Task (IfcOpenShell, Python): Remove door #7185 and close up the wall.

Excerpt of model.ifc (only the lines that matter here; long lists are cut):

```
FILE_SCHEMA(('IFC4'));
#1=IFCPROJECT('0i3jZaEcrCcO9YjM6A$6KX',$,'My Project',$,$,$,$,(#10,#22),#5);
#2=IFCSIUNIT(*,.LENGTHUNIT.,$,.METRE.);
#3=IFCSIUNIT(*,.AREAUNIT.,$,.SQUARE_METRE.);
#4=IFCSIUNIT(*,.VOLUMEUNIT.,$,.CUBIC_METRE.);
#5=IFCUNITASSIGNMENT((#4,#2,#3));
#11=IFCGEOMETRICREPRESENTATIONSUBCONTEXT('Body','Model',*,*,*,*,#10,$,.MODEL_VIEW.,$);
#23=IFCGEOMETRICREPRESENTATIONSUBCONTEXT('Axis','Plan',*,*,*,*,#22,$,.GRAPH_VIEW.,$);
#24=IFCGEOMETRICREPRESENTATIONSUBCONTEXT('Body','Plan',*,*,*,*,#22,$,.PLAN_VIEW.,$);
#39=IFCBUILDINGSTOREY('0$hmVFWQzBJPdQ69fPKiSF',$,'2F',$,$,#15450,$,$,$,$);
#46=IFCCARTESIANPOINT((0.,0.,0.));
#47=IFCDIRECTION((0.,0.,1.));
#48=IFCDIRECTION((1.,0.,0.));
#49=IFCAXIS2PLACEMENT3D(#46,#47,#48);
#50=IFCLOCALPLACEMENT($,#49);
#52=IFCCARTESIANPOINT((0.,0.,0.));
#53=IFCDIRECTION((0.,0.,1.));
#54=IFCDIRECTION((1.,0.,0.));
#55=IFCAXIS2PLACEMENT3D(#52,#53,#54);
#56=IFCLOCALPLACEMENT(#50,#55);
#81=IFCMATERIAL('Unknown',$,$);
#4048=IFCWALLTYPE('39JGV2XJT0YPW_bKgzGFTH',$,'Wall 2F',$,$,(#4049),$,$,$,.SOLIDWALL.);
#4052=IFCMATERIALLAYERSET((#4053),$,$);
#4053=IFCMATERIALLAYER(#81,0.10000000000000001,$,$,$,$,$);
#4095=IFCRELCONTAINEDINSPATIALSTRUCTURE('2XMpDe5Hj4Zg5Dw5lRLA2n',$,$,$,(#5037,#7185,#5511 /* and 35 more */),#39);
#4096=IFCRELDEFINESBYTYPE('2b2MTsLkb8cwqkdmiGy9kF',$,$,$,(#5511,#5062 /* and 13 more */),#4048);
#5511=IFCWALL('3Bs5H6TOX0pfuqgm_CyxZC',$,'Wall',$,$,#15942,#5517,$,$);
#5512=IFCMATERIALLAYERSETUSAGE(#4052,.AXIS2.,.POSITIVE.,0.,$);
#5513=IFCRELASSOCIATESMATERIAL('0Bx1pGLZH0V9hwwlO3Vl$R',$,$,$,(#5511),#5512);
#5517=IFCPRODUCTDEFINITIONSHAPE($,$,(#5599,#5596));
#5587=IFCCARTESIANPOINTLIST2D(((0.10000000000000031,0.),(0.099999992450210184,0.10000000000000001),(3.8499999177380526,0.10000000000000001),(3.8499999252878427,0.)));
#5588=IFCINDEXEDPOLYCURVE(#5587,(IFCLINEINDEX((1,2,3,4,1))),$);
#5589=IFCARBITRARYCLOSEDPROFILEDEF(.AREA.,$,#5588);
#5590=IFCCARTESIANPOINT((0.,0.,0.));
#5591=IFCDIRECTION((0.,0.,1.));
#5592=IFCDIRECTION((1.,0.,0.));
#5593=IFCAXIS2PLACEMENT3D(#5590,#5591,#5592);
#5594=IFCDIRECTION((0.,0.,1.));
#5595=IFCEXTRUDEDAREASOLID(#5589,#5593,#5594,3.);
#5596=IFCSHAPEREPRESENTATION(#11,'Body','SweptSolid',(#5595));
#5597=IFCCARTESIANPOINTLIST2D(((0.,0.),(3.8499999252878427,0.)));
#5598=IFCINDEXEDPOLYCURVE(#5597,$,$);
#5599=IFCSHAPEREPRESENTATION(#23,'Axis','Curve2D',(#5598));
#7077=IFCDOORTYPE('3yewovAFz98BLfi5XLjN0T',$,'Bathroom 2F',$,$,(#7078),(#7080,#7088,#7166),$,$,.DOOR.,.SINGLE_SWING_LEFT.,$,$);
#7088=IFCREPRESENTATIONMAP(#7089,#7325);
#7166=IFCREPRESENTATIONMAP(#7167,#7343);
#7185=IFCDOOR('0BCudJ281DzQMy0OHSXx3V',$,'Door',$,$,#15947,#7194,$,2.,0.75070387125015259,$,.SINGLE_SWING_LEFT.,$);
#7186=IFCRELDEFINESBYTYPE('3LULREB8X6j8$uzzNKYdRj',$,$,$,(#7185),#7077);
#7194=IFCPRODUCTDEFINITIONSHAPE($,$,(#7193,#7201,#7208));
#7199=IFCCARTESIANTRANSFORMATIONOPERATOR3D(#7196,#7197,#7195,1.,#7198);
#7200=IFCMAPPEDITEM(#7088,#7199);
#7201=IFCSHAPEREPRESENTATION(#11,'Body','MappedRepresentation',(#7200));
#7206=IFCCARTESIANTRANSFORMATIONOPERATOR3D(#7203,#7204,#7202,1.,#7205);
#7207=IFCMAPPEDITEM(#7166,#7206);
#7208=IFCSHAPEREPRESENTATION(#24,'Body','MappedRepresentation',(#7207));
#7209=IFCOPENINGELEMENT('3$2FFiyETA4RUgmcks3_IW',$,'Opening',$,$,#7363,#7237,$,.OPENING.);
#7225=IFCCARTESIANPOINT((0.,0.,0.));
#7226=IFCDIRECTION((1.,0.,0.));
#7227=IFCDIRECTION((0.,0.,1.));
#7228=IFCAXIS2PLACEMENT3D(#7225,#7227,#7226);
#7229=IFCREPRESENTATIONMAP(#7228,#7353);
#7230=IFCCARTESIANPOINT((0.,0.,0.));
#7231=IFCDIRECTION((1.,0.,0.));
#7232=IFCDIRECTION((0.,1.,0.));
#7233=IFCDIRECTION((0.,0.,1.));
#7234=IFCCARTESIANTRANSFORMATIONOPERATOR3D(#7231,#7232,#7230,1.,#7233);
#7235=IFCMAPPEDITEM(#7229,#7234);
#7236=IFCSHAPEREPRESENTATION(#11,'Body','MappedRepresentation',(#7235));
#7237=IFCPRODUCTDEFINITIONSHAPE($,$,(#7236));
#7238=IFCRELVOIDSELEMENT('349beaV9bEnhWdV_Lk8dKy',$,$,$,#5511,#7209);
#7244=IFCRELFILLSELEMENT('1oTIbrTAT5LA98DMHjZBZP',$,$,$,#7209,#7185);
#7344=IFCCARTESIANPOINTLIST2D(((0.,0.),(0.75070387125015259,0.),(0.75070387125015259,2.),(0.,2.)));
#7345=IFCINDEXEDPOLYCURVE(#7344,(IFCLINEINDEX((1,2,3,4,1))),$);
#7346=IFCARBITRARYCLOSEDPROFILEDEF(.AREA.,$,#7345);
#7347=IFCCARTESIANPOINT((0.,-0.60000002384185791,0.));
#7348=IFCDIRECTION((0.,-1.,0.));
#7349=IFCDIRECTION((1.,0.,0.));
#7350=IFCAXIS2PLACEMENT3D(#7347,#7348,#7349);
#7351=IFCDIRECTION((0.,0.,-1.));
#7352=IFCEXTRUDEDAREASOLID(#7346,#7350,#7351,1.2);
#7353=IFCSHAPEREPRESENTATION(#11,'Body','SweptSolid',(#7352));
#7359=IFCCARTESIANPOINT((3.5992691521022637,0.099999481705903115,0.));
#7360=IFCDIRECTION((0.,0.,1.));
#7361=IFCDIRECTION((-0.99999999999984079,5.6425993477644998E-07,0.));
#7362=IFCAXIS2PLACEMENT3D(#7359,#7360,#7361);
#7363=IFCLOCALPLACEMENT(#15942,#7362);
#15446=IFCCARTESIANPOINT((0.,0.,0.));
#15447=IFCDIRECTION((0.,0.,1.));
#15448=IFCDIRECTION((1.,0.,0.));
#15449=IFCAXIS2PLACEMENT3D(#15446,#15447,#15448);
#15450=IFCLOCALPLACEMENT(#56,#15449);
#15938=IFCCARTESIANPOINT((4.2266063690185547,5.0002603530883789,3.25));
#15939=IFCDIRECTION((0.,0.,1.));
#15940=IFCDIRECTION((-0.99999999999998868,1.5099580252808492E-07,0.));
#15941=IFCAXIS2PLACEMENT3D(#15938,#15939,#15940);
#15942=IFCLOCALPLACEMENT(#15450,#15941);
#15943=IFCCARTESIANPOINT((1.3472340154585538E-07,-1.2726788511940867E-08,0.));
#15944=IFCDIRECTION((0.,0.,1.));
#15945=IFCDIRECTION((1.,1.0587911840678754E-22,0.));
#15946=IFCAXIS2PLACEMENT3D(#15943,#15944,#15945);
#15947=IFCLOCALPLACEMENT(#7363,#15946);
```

```python
import ifcopenshell
import ifcopenshell.api.feature
import ifcopenshell.api.root
import ifcopenshell.geom
import ifcopenshell.util.shape

model = ifcopenshell.open("model.ifc")
settings = ifcopenshell.geom.settings()


def volume(element):
    """Net volume in cubic metres, openings subtracted."""
    shape = ifcopenshell.geom.create_shape(settings, element)
    return ifcopenshell.util.shape.get_volume(shape.geometry)


door = model.by_guid("0BCudJ281DzQMy0OHSXx3V")
opening = door.FillsVoids[0].RelatingOpeningElement
wall = opening.VoidsElements[0].RelatingBuildingElement
before = volume(wall)

ifcopenshell.api.root.remove_product(model, product=door)
ifcopenshell.api.feature.remove_feature(model, feature=opening)

after = volume(wall)

print(f"wall volume {before:.3f} -> {after:.3f} m3")

model.write("model_rev.ifc")
```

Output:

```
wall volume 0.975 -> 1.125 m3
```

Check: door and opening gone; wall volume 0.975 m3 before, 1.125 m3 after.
